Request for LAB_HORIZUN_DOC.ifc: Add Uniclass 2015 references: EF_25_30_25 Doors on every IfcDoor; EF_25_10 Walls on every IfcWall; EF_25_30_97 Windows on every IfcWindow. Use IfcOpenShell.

First a look at what the model holds.

```python
import ifcopenshell

model = ifcopenshell.open("LAB_HORIZUN_DOC.ifc")
print(model.schema)
print("classifications:", [c.Name for c in model.by_type("IfcClassification")])
for ifc_class in ("IfcDoor", "IfcRoof", "IfcStair", "IfcWall", "IfcWindow"):
    print(ifc_class, len(model.by_type(ifc_class)))
```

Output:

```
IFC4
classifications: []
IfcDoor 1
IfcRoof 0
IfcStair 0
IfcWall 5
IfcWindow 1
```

```python
import ifcopenshell
import ifcopenshell.api.classification

model = ifcopenshell.open("LAB_HORIZUN_DOC.ifc")

system = ifcopenshell.api.classification.add_classification(model, classification="Uniclass 2015")

codes = {
    "IfcDoor": ("EF_25_30_25", "Doors"),
    "IfcWall": ("EF_25_10", "Walls"),
    "IfcWindow": ("EF_25_30_97", "Windows"),
}
for ifc_class, (code, name) in codes.items():
    products = model.by_type(ifc_class)
    ifcopenshell.api.classification.add_reference(
        model, products=products, classification=system, identification=code, name=name
    )
    print(code, len(products))

model.write("LAB_HORIZUN_DOC-out.ifc")
```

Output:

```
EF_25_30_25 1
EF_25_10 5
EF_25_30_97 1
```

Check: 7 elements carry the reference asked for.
